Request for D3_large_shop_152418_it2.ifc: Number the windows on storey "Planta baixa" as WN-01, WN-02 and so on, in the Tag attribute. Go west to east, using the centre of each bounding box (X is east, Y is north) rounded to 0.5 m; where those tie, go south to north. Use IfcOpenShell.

First a look at what the model holds.

```python
import ifcopenshell
import ifcopenshell.util.element
import ifcopenshell.util.placement

model = ifcopenshell.open("D3_large_shop_152418_it2.ifc")
print(model.schema)
storey = next(s for s in model.by_type("IfcBuildingStorey") if s.Name == "Planta baixa")
windows = [e for e in ifcopenshell.util.element.get_decomposition(storey) if e.is_a("IfcWindow")]
for e in sorted(windows, key=lambda e: e.id()):
    origin = ifcopenshell.util.placement.get_local_placement(e.ObjectPlacement)[:3, 3]
    print(e.id(), e.Tag, e.Name, origin.round(2) + 0.0, sep=" | ")
```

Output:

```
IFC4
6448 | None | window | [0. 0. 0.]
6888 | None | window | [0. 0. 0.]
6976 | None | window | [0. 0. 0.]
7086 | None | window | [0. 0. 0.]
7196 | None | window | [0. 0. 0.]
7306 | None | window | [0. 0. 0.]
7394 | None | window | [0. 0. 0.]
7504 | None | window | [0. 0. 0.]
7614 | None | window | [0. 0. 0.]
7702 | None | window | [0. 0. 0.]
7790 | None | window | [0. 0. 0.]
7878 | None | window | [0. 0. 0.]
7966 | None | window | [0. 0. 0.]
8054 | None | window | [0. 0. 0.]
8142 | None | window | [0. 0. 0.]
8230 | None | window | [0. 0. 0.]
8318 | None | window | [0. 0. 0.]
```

```python
import ifcopenshell
import ifcopenshell.geom
import ifcopenshell.util.element
import ifcopenshell.util.shape

model = ifcopenshell.open("D3_large_shop_152418_it2.ifc")
settings = ifcopenshell.geom.settings()
settings.set("use-world-coords", True)


def centre(element):
    shape = ifcopenshell.geom.create_shape(settings, element)
    return ifcopenshell.util.shape.get_bbox_centroid(shape.geometry)


storey = next(s for s in model.by_type("IfcBuildingStorey") if s.Name == "Planta baixa")
windows = [e for e in ifcopenshell.util.element.get_decomposition(storey) if e.is_a("IfcWindow")]

# Insertion points can sit at a corner or the storey origin, so sort by the geometry (in metres).
centres = {e: centre(e) for e in windows}
windows.sort(key=lambda e: (round(centres[e][0] / 0.5), centres[e][1]))

for i, e in enumerate(windows, start=1):
    number = f"WN-{i:02d}"
    e.Tag = number
    print(e.id(), number)

model.write("D3_large_shop_152418_it2-out.ifc")
```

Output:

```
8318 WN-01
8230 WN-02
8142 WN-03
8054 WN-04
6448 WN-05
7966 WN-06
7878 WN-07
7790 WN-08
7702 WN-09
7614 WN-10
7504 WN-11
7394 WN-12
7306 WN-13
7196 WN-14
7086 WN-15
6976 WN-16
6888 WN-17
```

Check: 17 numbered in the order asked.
